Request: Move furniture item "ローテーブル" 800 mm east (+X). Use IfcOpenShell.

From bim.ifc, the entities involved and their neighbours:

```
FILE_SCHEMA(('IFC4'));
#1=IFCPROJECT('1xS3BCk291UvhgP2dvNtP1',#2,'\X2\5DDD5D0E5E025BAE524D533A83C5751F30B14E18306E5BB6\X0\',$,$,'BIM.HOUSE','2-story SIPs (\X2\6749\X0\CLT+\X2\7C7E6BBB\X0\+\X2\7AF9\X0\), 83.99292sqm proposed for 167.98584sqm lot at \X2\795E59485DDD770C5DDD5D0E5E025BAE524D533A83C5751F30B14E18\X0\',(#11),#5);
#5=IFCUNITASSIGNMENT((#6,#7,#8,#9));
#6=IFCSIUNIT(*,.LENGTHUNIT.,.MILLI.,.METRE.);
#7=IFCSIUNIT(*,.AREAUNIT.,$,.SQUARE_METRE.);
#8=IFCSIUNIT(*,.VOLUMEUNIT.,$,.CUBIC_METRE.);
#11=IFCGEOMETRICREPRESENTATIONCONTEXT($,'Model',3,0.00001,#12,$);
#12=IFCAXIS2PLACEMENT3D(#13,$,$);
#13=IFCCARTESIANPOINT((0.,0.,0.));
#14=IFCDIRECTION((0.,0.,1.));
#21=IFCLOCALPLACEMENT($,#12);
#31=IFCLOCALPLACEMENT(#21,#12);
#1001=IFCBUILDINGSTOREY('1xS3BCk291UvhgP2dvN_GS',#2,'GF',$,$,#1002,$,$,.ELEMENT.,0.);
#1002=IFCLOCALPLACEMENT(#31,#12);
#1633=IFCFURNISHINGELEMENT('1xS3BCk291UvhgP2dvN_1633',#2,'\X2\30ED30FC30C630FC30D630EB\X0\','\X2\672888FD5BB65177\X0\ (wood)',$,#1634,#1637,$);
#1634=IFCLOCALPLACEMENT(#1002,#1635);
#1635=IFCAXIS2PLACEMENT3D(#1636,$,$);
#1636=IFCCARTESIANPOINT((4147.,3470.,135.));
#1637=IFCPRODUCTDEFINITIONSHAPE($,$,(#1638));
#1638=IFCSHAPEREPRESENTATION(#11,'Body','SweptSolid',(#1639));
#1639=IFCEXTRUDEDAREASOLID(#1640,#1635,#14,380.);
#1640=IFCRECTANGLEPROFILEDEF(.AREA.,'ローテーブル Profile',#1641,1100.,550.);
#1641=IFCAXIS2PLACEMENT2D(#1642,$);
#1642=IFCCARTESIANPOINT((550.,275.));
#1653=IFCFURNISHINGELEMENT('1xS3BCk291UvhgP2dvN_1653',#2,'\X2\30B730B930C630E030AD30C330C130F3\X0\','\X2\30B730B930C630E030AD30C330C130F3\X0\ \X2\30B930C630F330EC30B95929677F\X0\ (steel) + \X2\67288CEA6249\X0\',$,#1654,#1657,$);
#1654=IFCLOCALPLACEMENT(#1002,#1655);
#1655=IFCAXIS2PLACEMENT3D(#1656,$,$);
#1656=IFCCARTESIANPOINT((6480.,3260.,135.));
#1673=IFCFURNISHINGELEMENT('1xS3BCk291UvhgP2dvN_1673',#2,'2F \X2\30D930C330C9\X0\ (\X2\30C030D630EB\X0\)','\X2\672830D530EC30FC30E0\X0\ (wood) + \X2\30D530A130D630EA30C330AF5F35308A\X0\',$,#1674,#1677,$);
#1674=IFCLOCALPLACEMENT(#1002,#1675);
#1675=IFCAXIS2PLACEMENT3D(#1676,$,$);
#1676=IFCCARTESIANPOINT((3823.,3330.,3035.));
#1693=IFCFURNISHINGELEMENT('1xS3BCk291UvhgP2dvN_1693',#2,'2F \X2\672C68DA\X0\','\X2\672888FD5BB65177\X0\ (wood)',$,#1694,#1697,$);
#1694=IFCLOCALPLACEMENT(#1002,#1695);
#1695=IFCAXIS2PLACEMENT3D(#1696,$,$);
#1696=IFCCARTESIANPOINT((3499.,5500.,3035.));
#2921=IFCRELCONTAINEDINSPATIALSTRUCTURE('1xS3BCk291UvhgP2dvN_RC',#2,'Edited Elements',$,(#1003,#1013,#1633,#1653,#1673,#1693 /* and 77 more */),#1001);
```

```python
import ifcopenshell
import ifcopenshell.api.geometry
import ifcopenshell.util.placement

model = ifcopenshell.open("bim.ifc")

item = model.by_guid("1xS3BCk291UvhgP2dvN_1633")
matrix = ifcopenshell.util.placement.get_local_placement(item.ObjectPlacement)
matrix[0, 3] += 800.0
ifcopenshell.api.geometry.edit_object_placement(model, product=item, matrix=matrix, is_si=False)

print(ifcopenshell.util.placement.get_local_placement(item.ObjectPlacement).round(3) + 0.0)

model.write("bim_rev.ifc")
```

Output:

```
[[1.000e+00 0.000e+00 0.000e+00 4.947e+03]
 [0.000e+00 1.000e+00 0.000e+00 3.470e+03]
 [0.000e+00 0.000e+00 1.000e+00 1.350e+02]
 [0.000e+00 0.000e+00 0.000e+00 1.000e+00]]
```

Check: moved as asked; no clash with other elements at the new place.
